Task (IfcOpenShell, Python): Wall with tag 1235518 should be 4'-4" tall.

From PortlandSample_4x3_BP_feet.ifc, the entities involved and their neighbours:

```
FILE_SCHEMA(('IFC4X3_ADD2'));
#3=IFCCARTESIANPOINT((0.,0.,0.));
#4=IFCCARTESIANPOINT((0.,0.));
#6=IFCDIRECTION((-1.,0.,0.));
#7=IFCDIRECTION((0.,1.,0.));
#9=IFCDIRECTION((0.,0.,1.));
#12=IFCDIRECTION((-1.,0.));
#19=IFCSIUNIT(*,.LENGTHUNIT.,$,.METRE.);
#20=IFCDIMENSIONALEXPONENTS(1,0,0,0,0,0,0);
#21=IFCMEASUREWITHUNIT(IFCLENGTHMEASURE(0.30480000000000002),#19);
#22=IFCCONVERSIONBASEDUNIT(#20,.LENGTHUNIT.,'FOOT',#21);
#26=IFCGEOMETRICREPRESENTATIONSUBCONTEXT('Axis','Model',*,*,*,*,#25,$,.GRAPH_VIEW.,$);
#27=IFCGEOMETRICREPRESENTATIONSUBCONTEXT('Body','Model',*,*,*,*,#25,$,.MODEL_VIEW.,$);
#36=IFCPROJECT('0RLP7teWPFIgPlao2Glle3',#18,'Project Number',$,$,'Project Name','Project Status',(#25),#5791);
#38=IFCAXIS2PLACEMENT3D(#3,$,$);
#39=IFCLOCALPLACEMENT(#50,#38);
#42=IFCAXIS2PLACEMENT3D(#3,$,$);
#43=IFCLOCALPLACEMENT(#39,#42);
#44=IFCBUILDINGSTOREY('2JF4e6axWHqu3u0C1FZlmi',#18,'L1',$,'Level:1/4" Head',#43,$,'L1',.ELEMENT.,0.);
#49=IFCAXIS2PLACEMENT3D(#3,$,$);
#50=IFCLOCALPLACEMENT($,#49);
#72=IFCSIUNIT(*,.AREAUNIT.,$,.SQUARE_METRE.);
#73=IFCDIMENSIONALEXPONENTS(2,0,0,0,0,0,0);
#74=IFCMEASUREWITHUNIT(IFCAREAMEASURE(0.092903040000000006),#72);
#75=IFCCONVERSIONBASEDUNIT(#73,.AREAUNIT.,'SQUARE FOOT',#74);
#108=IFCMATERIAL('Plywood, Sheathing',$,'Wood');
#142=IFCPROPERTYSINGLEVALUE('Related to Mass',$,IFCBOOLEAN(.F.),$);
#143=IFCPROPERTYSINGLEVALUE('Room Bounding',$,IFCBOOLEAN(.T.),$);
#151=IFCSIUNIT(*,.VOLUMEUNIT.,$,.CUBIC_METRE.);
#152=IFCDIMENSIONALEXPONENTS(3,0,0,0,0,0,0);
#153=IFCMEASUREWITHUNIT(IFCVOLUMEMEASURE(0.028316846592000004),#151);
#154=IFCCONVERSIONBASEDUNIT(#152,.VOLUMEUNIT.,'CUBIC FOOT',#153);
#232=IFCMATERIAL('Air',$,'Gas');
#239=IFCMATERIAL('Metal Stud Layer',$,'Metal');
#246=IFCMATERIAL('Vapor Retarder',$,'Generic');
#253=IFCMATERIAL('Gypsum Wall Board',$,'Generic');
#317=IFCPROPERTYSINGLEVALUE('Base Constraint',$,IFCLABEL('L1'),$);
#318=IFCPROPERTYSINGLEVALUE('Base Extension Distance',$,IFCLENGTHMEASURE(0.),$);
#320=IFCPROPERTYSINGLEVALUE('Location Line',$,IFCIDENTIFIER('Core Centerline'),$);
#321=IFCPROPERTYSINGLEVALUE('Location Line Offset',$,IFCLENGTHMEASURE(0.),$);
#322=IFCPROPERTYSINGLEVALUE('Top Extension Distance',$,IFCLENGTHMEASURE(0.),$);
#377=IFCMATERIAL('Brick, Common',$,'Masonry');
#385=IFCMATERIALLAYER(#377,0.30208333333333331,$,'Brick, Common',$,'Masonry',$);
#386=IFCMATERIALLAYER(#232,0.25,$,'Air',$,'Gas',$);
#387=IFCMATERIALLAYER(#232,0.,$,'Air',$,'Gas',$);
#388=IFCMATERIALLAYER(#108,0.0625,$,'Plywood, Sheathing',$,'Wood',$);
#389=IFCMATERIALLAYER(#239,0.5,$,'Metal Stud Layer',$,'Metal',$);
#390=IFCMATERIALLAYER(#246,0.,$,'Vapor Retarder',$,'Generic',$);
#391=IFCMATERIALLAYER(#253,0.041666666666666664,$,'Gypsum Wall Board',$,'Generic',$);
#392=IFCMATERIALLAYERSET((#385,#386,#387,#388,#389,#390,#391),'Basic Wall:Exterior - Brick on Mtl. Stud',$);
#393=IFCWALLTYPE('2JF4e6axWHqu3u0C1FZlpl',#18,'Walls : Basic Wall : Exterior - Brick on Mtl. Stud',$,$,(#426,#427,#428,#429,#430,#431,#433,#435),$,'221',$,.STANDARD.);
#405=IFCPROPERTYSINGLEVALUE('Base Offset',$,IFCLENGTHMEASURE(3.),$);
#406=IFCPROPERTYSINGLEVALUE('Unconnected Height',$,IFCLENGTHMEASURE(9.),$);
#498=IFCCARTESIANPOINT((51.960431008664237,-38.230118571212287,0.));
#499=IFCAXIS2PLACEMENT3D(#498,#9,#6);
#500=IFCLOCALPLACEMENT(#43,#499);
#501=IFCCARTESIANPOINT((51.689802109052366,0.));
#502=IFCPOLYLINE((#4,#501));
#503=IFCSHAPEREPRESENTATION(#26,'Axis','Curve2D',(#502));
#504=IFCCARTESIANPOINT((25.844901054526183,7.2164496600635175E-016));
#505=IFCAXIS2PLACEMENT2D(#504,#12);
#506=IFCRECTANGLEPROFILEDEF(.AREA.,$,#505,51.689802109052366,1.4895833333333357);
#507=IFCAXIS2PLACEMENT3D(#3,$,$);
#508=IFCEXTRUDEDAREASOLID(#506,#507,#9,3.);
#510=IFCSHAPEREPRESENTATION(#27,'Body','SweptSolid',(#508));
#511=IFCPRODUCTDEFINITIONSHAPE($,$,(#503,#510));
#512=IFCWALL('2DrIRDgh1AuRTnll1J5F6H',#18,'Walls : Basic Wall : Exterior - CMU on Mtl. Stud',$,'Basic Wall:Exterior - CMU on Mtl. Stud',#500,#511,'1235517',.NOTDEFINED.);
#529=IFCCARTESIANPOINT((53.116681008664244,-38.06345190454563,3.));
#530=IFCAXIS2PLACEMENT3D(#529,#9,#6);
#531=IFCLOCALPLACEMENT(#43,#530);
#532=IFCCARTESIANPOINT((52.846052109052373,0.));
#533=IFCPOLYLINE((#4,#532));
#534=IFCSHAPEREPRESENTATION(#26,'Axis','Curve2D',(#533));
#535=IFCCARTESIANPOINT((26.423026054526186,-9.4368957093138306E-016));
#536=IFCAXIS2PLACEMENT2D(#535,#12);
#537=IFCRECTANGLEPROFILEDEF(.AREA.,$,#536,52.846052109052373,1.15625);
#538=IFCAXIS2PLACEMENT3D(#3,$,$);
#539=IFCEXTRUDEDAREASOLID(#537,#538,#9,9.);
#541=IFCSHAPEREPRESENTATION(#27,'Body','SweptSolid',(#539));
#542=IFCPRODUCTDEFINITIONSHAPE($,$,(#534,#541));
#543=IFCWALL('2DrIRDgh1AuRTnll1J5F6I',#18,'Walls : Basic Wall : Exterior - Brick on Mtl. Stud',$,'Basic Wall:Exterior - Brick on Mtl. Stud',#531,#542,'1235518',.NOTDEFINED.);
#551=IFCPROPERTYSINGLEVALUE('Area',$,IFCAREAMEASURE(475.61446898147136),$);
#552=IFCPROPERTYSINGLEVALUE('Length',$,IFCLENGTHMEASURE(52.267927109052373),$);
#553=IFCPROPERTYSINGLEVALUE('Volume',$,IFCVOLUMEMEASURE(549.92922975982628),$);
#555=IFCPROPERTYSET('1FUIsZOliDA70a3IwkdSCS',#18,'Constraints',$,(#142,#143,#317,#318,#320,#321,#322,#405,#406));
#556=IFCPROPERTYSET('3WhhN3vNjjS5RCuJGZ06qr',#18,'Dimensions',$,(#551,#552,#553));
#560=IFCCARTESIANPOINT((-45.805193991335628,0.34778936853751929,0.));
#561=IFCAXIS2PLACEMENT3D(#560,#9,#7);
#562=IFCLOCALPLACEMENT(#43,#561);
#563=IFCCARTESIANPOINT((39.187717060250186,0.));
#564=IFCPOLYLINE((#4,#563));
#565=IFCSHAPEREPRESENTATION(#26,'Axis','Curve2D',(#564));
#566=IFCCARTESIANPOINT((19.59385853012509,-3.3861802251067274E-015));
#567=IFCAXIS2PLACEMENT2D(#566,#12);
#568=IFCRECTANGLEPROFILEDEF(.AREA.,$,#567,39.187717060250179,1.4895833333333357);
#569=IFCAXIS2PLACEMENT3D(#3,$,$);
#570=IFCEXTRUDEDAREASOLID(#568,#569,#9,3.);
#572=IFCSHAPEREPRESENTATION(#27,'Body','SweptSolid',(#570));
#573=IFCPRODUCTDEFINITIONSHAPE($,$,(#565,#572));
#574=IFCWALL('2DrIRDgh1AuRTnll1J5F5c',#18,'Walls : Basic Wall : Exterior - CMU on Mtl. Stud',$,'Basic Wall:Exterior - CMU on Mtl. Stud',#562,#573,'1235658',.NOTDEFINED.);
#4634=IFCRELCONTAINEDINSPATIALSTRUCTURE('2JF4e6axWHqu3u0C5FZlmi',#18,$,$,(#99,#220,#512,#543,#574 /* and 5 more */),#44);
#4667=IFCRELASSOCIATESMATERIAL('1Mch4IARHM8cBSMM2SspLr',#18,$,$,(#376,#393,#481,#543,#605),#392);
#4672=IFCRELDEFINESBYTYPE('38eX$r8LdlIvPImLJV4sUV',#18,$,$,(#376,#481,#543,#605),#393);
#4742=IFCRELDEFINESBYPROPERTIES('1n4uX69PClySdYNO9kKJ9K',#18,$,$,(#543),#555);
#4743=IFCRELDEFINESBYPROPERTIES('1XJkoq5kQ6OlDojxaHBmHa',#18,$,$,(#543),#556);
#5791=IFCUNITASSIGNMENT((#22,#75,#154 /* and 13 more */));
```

```python
import ifcopenshell
import ifcopenshell.api.pset
import ifcopenshell.geom
import ifcopenshell.util.element
import ifcopenshell.util.representation
import ifcopenshell.util.shape
import ifcopenshell.util.unit

model = ifcopenshell.open("PortlandSample_4x3_BP_feet.ifc")
unit_scale = ifcopenshell.util.unit.calculate_unit_scale(model)
area_scale = ifcopenshell.util.unit.calculate_unit_scale(model, "AREAUNIT")
volume_scale = ifcopenshell.util.unit.calculate_unit_scale(model, "VOLUMEUNIT")
settings = ifcopenshell.geom.settings()


def volume(element):
    """Net volume in cubic metres, openings subtracted."""
    shape = ifcopenshell.geom.create_shape(settings, element)
    return ifcopenshell.util.shape.get_volume(shape.geometry)


wall = model.by_id(543)
before = volume(wall)

body = ifcopenshell.util.representation.get_representation(wall, "Model", "Body")
solid = body.Items[0]
old_height = solid.Depth
solid.Depth = 52 * 0.0254 / unit_scale
after = volume(wall)
thickness = 0.3524  # wall thickness in metres

# Update the stored height, areas and volumes.
pset = model.by_id(ifcopenshell.util.element.get_pset(wall, "Constraints", should_inherit=False)["id"])
ifcopenshell.api.pset.edit_pset(model, pset=pset, properties={
    "Unconnected Height": model.create_entity("IfcLengthMeasure", solid.Depth),
})
pset = model.by_id(ifcopenshell.util.element.get_pset(wall, "Dimensions", should_inherit=False)["id"])
ifcopenshell.api.pset.edit_pset(model, pset=pset, properties={
    "Area": model.create_entity("IfcAreaMeasure", after / thickness / area_scale),
    "Volume": model.create_entity("IfcVolumeMeasure", after / volume_scale),
})

print(f"height {old_height:g} -> {solid.Depth:g}, volume {before:.3f} -> {after:.3f} m3")

model.write("PortlandSample_4x3_BP_feet-out.ifc")
```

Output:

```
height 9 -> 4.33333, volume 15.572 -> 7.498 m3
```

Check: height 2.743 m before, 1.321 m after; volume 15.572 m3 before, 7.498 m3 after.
